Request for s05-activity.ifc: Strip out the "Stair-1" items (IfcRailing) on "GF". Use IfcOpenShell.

First a look at what the model holds.

```python
import ifcopenshell
import ifcopenshell.util.element

model = ifcopenshell.open("s05-activity.ifc")
print(model.schema)
storey = next(s for s in model.by_type("IfcBuildingStorey") if s.Name == "GF")
railings = [e for e in ifcopenshell.util.element.get_decomposition(storey) if e.is_a("IfcRailing")]
seen = {}
for e in railings:
    element_type = ifcopenshell.util.element.get_type(e)
    name = element_type.Name if element_type not in (None, e) else None
    seen[name] = seen.get(name, 0) + 1
for name, count in sorted(seen.items(), key=str):
    print(count, "x", name)
```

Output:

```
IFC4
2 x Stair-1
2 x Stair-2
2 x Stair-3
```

```python
import ifcopenshell
import ifcopenshell.api.root
import ifcopenshell.util.element

model = ifcopenshell.open("s05-activity.ifc")

storey = next(s for s in model.by_type("IfcBuildingStorey") if s.Name == "GF")
railings = [e for e in ifcopenshell.util.element.get_decomposition(storey) if e.is_a("IfcRailing")]
targets = [e for e in railings if (t := ifcopenshell.util.element.get_type(e)) not in (None, e) and t.Name == "Stair-1"]

for e in targets:
    ifcopenshell.api.root.remove_product(model, product=e)
print(len(targets), "removed")

model.write("s05-activity_updated.ifc")
```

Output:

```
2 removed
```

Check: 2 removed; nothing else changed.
